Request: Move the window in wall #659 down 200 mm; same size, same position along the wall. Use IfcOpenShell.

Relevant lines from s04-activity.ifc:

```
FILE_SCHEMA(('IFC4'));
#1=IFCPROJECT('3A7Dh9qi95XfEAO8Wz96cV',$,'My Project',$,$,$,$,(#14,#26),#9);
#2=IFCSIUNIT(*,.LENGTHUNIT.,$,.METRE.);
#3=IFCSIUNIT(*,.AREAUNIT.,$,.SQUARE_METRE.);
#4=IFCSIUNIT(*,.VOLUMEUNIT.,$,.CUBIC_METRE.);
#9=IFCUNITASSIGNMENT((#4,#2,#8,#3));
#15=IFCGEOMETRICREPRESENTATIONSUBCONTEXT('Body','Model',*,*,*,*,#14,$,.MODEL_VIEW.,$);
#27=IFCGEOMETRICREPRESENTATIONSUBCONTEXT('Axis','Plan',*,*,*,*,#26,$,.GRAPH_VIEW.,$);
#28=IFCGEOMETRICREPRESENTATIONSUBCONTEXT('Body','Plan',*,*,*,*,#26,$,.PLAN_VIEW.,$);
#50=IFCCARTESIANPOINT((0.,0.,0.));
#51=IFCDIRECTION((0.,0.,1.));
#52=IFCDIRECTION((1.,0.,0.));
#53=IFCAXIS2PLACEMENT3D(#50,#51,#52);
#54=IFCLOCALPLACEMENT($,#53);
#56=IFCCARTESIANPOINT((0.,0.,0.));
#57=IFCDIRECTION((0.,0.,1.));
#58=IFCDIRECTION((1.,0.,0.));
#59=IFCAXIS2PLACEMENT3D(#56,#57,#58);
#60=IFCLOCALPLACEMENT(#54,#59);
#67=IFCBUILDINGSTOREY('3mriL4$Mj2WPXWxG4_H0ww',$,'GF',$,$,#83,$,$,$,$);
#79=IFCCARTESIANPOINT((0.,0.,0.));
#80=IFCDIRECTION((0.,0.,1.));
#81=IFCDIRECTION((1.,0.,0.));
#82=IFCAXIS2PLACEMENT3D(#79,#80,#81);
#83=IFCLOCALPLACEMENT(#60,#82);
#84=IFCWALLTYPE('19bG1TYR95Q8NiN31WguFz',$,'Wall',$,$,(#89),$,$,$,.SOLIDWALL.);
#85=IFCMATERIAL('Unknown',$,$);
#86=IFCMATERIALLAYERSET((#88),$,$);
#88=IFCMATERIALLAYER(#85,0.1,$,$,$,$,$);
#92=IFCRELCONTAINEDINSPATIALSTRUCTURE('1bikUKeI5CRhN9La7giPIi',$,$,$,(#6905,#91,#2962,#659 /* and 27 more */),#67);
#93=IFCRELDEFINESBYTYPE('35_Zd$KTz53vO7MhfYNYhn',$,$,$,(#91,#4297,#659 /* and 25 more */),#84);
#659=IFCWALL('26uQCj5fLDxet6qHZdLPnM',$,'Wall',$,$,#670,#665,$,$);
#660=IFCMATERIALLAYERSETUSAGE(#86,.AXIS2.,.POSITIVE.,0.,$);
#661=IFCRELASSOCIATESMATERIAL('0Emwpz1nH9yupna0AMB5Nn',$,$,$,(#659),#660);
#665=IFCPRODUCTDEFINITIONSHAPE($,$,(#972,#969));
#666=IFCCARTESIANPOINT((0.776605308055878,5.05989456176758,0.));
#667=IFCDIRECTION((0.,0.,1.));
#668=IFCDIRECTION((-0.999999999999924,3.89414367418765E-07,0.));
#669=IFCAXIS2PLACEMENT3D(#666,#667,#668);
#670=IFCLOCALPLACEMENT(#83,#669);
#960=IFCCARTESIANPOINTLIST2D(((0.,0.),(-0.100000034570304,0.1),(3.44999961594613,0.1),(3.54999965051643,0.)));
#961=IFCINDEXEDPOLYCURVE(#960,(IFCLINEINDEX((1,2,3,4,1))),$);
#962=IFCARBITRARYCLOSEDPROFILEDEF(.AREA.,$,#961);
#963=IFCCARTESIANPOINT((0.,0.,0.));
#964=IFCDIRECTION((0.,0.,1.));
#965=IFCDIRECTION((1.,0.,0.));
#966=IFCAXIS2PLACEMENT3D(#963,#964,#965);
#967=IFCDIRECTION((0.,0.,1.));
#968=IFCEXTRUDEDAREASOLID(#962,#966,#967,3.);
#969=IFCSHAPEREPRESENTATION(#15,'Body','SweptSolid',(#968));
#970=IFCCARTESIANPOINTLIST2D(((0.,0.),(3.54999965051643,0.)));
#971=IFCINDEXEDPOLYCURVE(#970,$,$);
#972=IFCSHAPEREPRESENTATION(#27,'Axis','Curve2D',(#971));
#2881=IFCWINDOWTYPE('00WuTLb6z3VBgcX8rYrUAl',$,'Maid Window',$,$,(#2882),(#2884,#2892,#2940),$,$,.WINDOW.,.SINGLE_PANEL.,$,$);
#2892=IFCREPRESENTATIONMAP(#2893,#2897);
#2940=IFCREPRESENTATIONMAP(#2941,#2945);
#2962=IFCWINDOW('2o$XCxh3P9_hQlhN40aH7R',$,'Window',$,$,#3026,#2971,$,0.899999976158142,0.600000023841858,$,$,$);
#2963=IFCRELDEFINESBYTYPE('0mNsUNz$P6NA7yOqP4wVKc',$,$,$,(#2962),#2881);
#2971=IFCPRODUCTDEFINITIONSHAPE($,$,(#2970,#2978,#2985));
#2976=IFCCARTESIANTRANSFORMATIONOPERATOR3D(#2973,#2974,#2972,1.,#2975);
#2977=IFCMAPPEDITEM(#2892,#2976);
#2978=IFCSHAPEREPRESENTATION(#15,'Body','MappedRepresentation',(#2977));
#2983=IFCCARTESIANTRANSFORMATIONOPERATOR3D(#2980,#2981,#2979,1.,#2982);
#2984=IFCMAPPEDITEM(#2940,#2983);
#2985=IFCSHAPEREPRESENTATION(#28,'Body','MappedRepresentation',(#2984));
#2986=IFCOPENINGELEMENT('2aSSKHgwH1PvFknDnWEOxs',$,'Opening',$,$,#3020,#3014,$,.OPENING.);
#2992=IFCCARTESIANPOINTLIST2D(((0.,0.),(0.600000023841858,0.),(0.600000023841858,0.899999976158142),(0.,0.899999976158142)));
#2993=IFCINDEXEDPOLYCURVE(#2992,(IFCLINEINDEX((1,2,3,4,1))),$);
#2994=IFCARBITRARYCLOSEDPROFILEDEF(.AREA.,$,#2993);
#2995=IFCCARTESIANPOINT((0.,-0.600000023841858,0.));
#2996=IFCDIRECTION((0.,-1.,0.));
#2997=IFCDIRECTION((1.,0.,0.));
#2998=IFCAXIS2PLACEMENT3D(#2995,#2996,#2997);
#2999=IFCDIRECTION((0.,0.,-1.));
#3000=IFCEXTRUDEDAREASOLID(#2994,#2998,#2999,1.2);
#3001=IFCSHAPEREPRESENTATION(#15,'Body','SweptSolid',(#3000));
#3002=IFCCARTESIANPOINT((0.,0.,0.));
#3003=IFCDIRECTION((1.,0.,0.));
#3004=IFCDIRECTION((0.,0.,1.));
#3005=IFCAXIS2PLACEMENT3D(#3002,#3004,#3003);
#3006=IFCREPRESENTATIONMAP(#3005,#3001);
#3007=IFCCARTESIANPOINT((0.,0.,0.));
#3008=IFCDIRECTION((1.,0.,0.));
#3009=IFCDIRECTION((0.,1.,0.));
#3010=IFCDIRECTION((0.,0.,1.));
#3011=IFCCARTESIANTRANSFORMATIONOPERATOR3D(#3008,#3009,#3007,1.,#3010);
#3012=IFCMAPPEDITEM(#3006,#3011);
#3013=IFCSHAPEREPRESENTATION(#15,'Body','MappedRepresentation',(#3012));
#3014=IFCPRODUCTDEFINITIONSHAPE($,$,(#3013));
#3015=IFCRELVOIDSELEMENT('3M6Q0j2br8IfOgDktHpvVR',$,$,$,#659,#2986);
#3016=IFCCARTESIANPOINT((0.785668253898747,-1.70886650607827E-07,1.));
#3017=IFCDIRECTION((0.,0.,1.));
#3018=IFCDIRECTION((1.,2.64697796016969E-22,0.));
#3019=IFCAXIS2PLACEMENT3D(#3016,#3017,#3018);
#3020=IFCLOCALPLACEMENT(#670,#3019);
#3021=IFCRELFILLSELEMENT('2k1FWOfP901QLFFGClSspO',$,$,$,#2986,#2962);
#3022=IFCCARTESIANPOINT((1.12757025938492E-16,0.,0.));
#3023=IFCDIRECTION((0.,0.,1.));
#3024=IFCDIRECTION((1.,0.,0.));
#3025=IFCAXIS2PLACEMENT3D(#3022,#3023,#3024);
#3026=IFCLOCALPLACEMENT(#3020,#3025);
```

```python
import numpy as np
import ifcopenshell
import ifcopenshell.api.geometry
import ifcopenshell.util.placement
import ifcopenshell.util.unit

model = ifcopenshell.open("s04-activity.ifc")
unit_scale = ifcopenshell.util.unit.calculate_unit_scale(model)

window = model.by_guid("2o$XCxh3P9_hQlhN40aH7R")
opening = window.FillsVoids[0].RelatingOpeningElement
dz = -0.2 / unit_scale

shift = np.array([0.0, 0.0, dz])
# The window is placed relative to its opening, so it follows when the opening moves.
matrix = ifcopenshell.util.placement.get_local_placement(opening.ObjectPlacement)
matrix[:3, 3] += shift
ifcopenshell.api.geometry.edit_object_placement(
    model, product=opening, matrix=matrix, is_si=False, should_transform_children=True
)

print(f"moved by {dz * unit_scale:+.3f} m")

model.write("s04-activity_v2.ifc")
```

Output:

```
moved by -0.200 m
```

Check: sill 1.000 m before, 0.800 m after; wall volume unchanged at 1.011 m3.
